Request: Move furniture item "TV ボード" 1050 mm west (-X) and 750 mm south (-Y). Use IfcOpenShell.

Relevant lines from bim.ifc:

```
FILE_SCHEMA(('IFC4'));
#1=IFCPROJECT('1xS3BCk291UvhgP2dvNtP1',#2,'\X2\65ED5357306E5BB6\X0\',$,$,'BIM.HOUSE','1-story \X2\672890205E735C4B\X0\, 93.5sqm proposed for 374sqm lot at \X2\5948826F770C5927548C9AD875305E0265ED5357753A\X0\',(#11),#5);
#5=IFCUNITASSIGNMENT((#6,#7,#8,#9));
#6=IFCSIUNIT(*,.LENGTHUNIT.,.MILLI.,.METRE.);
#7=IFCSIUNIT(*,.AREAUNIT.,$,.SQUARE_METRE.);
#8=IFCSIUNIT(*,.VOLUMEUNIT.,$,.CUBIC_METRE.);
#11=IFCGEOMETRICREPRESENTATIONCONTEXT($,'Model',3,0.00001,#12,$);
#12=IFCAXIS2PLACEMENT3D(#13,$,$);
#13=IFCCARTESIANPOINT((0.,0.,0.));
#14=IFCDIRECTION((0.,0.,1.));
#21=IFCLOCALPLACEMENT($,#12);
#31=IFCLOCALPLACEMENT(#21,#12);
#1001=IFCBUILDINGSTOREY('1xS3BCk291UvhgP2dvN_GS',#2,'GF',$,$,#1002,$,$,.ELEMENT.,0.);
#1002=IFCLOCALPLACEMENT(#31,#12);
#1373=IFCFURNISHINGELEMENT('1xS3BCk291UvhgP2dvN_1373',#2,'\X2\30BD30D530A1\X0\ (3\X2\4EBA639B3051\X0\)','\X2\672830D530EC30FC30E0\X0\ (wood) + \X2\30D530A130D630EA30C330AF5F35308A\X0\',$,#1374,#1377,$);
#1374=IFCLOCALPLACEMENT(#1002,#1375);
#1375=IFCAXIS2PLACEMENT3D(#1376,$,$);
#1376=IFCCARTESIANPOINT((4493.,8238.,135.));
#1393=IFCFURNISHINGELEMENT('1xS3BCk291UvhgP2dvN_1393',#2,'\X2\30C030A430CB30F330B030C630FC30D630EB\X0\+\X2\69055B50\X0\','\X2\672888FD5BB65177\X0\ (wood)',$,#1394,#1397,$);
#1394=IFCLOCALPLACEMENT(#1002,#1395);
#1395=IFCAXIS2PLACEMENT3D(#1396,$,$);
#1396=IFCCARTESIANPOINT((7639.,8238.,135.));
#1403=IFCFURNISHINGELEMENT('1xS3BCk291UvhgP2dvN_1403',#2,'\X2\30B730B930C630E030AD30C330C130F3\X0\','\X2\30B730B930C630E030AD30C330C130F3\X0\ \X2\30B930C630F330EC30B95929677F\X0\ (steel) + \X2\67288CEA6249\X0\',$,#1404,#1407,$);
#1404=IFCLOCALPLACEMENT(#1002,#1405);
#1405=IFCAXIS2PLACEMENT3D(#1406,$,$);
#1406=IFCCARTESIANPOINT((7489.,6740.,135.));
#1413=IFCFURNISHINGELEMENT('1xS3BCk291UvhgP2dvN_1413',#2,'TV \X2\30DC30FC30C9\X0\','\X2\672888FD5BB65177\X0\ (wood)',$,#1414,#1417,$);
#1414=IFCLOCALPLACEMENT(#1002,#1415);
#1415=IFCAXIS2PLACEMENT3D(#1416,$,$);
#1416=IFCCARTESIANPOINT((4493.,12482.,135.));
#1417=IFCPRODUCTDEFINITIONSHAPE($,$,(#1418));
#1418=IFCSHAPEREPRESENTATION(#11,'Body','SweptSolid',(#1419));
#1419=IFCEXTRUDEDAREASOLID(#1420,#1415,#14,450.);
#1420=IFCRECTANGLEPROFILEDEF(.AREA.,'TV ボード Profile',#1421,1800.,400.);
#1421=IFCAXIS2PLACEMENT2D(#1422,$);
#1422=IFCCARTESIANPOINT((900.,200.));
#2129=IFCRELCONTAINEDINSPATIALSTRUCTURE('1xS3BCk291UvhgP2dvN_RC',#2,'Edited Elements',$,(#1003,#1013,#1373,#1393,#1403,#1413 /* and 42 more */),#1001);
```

```python
import ifcopenshell
import ifcopenshell.api.geometry
import ifcopenshell.util.placement
import ifcopenshell.util.unit

model = ifcopenshell.open("bim.ifc")
unit_scale = ifcopenshell.util.unit.calculate_unit_scale(model)

item = model.by_guid("1xS3BCk291UvhgP2dvN_1413")
matrix = ifcopenshell.util.placement.get_local_placement(item.ObjectPlacement)
matrix[0, 3] -= 1.05 / unit_scale
matrix[1, 3] -= 0.75 / unit_scale
ifcopenshell.api.geometry.edit_object_placement(model, product=item, matrix=matrix, is_si=False)

print(ifcopenshell.util.placement.get_local_placement(item.ObjectPlacement).round(3) + 0.0)

model.write("bim_edited.ifc")
```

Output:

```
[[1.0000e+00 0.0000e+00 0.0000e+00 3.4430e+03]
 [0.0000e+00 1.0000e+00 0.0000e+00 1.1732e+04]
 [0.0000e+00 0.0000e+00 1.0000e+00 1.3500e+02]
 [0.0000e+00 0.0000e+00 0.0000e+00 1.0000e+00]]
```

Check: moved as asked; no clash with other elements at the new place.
